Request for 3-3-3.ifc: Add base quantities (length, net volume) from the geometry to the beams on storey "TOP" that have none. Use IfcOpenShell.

First a look at what the model holds.

```python
import ifcopenshell
import ifcopenshell.util.element
import ifcopenshell.util.unit

model = ifcopenshell.open("3-3-3.ifc")
print(model.schema)
for unit_type in ("LENGTHUNIT", "AREAUNIT", "VOLUMEUNIT"):
    print(unit_type, ifcopenshell.util.unit.calculate_unit_scale(model, unit_type))
storey = next(s for s in model.by_type("IfcBuildingStorey") if s.Name == "TOP")
beams = [e for e in ifcopenshell.util.element.get_decomposition(storey) if e.is_a("IfcBeam")]
for e in sorted(beams, key=lambda e: e.id()):
    print(e.id(), e.is_a(), e.Name, list(ifcopenshell.util.element.get_psets(e, qtos_only=True)), sep=" | ")
```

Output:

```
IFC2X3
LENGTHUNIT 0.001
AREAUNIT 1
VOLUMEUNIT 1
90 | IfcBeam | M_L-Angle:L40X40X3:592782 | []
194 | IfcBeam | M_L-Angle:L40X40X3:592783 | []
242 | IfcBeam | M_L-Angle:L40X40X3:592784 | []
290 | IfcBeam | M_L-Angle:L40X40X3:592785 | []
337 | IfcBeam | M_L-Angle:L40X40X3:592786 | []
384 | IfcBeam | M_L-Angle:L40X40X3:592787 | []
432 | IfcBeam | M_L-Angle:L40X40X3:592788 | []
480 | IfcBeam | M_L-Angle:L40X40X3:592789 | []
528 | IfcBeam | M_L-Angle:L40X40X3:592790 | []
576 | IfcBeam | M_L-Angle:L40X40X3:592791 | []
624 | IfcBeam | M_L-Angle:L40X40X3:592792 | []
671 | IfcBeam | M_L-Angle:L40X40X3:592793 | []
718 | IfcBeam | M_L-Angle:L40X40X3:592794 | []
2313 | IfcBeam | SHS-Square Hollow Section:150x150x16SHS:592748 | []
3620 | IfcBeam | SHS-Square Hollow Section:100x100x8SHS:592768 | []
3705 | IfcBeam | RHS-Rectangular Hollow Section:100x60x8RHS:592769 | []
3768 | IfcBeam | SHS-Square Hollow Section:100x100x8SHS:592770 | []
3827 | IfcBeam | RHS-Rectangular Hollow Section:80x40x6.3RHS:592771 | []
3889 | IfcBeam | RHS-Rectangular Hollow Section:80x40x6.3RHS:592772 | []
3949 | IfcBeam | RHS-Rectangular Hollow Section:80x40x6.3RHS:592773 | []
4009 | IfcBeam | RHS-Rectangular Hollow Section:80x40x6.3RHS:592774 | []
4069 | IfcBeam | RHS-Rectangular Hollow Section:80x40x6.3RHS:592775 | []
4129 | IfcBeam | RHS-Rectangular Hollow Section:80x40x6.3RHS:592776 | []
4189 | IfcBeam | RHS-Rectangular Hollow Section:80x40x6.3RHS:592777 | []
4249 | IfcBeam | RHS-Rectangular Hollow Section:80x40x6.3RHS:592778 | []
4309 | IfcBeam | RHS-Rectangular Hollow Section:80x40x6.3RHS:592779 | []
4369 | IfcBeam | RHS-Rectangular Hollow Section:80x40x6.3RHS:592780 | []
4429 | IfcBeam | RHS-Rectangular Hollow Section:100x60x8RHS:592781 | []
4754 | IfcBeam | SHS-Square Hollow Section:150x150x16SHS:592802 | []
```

```python
import ifcopenshell
import ifcopenshell.api.pset
import ifcopenshell.geom
import ifcopenshell.util.element
import ifcopenshell.util.shape
import ifcopenshell.util.unit

model = ifcopenshell.open("3-3-3.ifc")
unit_scale = ifcopenshell.util.unit.calculate_unit_scale(model)
volume_scale = ifcopenshell.util.unit.calculate_unit_scale(model, "VOLUMEUNIT")
settings = ifcopenshell.geom.settings()

storey = next(s for s in model.by_type("IfcBuildingStorey") if s.Name == "TOP")
beams = [e for e in ifcopenshell.util.element.get_decomposition(storey) if e.is_a("IfcBeam")]

for e in sorted(beams, key=lambda e: e.id()):
    if ifcopenshell.util.element.get_psets(e, qtos_only=True, should_inherit=False):
        continue
    # Geometry comes back in metres, in the element's own axes.
    shape = ifcopenshell.geom.create_shape(settings, e)
    values = {
        "Length": ifcopenshell.util.shape.get_max_xyz(shape.geometry) / unit_scale,
        "NetVolume": ifcopenshell.util.shape.get_volume(shape.geometry) / volume_scale,
    }
    qto = ifcopenshell.api.pset.add_qto(model, product=e, name="BaseQuantities")
    ifcopenshell.api.pset.edit_qto(model, qto=qto, properties=values)
    print(e.id(), {k: round(v, 3) for k, v in values.items()})

model.write("3-3-3_v2.ifc")
```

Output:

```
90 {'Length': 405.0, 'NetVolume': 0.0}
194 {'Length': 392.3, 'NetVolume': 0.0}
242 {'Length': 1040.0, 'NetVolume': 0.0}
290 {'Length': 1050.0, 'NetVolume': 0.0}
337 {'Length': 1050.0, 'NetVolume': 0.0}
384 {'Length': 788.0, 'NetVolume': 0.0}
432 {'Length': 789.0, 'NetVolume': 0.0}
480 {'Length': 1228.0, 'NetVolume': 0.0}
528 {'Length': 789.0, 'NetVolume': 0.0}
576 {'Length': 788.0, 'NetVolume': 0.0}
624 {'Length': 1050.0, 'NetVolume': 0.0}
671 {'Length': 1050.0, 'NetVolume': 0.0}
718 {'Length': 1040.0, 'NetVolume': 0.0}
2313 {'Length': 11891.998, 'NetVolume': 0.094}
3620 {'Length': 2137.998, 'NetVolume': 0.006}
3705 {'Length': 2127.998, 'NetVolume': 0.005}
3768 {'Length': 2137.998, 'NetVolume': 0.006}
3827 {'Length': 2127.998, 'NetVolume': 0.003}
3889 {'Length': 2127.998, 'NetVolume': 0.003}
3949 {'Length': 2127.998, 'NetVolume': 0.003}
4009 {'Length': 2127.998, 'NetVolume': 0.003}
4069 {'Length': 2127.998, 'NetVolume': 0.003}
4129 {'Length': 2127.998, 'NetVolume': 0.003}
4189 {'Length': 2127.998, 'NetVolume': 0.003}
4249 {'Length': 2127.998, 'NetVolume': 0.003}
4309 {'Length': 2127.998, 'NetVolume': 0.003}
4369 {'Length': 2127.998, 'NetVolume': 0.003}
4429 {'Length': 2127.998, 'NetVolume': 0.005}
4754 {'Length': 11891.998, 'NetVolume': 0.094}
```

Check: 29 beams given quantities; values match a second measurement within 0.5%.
